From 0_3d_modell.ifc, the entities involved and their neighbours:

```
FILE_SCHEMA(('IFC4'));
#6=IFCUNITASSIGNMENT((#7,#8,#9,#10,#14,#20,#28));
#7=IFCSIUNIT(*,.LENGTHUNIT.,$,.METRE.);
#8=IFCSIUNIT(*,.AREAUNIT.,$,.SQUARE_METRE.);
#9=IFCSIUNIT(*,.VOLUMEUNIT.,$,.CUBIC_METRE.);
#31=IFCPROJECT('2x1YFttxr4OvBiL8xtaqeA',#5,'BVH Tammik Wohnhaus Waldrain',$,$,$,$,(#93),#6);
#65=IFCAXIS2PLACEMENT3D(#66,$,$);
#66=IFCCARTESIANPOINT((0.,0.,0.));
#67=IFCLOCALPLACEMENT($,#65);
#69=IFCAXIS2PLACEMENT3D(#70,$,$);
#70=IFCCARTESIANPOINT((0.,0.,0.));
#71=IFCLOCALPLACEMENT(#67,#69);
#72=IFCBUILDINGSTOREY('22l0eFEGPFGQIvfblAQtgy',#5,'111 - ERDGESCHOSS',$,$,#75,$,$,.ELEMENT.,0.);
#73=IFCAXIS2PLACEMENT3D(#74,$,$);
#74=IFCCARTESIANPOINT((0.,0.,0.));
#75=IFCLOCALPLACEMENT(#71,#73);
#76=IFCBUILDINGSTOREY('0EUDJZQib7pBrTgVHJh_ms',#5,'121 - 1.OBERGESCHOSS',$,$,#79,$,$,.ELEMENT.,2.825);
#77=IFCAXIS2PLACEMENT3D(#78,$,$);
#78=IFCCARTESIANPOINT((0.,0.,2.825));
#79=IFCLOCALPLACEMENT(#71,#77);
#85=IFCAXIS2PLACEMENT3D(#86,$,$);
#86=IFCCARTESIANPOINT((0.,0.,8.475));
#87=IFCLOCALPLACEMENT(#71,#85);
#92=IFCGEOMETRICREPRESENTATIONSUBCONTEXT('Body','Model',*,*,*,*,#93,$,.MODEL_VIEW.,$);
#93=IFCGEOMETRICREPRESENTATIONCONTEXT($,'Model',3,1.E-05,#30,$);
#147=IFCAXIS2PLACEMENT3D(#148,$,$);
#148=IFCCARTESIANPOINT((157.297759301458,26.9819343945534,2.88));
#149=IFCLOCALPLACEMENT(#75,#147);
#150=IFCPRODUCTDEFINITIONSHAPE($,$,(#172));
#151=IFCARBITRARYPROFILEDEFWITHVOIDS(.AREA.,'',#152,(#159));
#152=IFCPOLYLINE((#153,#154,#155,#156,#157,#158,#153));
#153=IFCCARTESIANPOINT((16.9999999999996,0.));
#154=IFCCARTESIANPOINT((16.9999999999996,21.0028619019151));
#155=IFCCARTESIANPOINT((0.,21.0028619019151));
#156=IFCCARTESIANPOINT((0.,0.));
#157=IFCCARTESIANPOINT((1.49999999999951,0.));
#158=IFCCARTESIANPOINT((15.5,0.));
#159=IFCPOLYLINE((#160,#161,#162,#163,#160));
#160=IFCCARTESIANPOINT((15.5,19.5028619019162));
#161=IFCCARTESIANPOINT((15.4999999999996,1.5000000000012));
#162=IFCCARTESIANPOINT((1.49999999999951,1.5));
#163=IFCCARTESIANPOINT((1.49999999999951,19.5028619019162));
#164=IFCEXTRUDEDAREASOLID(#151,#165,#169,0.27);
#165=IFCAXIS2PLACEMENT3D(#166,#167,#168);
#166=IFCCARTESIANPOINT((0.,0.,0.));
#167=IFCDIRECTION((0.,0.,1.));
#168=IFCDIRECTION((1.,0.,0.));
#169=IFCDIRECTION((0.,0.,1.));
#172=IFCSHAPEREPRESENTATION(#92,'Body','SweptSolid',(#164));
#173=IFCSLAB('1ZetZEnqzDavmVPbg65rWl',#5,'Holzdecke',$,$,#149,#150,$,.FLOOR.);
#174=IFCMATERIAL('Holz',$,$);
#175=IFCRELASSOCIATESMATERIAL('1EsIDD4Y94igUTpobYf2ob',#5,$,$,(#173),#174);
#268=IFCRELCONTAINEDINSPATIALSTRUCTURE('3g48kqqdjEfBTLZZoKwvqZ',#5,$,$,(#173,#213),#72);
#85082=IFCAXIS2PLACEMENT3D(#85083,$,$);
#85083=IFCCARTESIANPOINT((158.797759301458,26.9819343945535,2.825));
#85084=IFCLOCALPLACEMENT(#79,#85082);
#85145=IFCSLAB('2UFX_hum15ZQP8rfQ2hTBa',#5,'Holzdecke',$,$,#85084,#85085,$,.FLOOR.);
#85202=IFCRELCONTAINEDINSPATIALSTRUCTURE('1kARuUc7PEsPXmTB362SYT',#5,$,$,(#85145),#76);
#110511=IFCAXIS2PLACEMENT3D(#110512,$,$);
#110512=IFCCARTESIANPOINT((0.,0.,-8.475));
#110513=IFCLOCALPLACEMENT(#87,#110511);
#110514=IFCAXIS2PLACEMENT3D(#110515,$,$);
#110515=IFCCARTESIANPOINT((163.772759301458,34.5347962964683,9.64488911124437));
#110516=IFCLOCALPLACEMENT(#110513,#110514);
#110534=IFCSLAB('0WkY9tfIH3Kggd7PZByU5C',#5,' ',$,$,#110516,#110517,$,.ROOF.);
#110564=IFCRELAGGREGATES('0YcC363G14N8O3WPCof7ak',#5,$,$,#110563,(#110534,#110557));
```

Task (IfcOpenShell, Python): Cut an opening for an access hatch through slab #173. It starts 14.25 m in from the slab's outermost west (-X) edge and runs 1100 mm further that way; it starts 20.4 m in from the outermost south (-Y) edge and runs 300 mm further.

```python
import numpy as np
import ifcopenshell
import ifcopenshell.api.feature
import ifcopenshell.api.geometry
import ifcopenshell.api.root
import ifcopenshell.geom
import ifcopenshell.util.placement
import ifcopenshell.util.representation
import ifcopenshell.util.shape
import ifcopenshell.util.unit

model = ifcopenshell.open("0_3d_modell.ifc")
unit_scale = ifcopenshell.util.unit.calculate_unit_scale(model)
settings = ifcopenshell.geom.settings()


def volume(element):
    """Net volume in cubic metres, openings subtracted."""
    shape = ifcopenshell.geom.create_shape(settings, element)
    return ifcopenshell.util.shape.get_volume(shape.geometry)


slab = model.by_guid("1ZetZEnqzDavmVPbg65rWl")
before = volume(slab)

# Extent in the slab's own axes, in metres. The edges named are its -X and -Y sides.
slab_shape = ifcopenshell.geom.create_shape(settings, slab)
vertices = ifcopenshell.util.shape.get_vertices(slab_shape.geometry)
x_min, y_min, bottom = vertices.min(axis=0)
top = vertices[:, 2].max()

opening = ifcopenshell.api.root.create_entity(model, ifc_class="IfcOpeningElement", name="Access hatch opening", predefined_type="OPENING")
context = ifcopenshell.util.representation.get_context(model, "Model", "Body", "MODEL_VIEW")
width, depth = 1.1, 0.3
outline = [(0.0, 0.0), (width, 0.0), (width, depth), (0.0, depth), (0.0, 0.0)]
# Overshoot both faces by 50 mm so the cut is clean.
shape = ifcopenshell.api.geometry.add_slab_representation(
    model, context=context, depth=top - bottom + 0.1, polyline=outline
)
ifcopenshell.api.geometry.assign_representation(model, product=opening, representation=shape)

matrix = ifcopenshell.util.placement.get_local_placement(slab.ObjectPlacement)
matrix[:, 3] = matrix @ np.append(np.array([x_min + 14.25, y_min + 20.4, bottom - 0.05]) / unit_scale, 1.0)
ifcopenshell.api.geometry.edit_object_placement(model, product=opening, matrix=matrix, is_si=False)
ifcopenshell.api.feature.add_feature(model, feature=opening, element=slab)

after = volume(slab)

print(f"slab volume {before:.3f} -> {after:.3f} m3")

model.write("0_3d_modell-out.ifc")
```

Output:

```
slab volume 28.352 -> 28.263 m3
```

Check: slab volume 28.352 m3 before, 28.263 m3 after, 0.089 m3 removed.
